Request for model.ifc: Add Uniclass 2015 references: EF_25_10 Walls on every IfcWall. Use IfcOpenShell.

First a look at what the model holds.

```python
import ifcopenshell

model = ifcopenshell.open("model.ifc")
print(model.schema)
print("classifications:", [c.Name for c in model.by_type("IfcClassification")])
for ifc_class in ("IfcDoor", "IfcRoof", "IfcStair", "IfcWall", "IfcWindow"):
    print(ifc_class, len(model.by_type(ifc_class)))
```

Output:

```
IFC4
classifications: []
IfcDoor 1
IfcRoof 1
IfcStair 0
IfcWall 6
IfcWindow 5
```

```python
import ifcopenshell
import ifcopenshell.api.classification

model = ifcopenshell.open("model.ifc")

system = ifcopenshell.api.classification.add_classification(model, classification="Uniclass 2015")

codes = {
    "IfcWall": ("EF_25_10", "Walls"),
}
for ifc_class, (code, name) in codes.items():
    products = model.by_type(ifc_class)
    ifcopenshell.api.classification.add_reference(
        model, products=products, classification=system, identification=code, name=name
    )
    print(code, len(products))

model.write("model_updated.ifc")
```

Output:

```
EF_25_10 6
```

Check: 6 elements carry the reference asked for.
